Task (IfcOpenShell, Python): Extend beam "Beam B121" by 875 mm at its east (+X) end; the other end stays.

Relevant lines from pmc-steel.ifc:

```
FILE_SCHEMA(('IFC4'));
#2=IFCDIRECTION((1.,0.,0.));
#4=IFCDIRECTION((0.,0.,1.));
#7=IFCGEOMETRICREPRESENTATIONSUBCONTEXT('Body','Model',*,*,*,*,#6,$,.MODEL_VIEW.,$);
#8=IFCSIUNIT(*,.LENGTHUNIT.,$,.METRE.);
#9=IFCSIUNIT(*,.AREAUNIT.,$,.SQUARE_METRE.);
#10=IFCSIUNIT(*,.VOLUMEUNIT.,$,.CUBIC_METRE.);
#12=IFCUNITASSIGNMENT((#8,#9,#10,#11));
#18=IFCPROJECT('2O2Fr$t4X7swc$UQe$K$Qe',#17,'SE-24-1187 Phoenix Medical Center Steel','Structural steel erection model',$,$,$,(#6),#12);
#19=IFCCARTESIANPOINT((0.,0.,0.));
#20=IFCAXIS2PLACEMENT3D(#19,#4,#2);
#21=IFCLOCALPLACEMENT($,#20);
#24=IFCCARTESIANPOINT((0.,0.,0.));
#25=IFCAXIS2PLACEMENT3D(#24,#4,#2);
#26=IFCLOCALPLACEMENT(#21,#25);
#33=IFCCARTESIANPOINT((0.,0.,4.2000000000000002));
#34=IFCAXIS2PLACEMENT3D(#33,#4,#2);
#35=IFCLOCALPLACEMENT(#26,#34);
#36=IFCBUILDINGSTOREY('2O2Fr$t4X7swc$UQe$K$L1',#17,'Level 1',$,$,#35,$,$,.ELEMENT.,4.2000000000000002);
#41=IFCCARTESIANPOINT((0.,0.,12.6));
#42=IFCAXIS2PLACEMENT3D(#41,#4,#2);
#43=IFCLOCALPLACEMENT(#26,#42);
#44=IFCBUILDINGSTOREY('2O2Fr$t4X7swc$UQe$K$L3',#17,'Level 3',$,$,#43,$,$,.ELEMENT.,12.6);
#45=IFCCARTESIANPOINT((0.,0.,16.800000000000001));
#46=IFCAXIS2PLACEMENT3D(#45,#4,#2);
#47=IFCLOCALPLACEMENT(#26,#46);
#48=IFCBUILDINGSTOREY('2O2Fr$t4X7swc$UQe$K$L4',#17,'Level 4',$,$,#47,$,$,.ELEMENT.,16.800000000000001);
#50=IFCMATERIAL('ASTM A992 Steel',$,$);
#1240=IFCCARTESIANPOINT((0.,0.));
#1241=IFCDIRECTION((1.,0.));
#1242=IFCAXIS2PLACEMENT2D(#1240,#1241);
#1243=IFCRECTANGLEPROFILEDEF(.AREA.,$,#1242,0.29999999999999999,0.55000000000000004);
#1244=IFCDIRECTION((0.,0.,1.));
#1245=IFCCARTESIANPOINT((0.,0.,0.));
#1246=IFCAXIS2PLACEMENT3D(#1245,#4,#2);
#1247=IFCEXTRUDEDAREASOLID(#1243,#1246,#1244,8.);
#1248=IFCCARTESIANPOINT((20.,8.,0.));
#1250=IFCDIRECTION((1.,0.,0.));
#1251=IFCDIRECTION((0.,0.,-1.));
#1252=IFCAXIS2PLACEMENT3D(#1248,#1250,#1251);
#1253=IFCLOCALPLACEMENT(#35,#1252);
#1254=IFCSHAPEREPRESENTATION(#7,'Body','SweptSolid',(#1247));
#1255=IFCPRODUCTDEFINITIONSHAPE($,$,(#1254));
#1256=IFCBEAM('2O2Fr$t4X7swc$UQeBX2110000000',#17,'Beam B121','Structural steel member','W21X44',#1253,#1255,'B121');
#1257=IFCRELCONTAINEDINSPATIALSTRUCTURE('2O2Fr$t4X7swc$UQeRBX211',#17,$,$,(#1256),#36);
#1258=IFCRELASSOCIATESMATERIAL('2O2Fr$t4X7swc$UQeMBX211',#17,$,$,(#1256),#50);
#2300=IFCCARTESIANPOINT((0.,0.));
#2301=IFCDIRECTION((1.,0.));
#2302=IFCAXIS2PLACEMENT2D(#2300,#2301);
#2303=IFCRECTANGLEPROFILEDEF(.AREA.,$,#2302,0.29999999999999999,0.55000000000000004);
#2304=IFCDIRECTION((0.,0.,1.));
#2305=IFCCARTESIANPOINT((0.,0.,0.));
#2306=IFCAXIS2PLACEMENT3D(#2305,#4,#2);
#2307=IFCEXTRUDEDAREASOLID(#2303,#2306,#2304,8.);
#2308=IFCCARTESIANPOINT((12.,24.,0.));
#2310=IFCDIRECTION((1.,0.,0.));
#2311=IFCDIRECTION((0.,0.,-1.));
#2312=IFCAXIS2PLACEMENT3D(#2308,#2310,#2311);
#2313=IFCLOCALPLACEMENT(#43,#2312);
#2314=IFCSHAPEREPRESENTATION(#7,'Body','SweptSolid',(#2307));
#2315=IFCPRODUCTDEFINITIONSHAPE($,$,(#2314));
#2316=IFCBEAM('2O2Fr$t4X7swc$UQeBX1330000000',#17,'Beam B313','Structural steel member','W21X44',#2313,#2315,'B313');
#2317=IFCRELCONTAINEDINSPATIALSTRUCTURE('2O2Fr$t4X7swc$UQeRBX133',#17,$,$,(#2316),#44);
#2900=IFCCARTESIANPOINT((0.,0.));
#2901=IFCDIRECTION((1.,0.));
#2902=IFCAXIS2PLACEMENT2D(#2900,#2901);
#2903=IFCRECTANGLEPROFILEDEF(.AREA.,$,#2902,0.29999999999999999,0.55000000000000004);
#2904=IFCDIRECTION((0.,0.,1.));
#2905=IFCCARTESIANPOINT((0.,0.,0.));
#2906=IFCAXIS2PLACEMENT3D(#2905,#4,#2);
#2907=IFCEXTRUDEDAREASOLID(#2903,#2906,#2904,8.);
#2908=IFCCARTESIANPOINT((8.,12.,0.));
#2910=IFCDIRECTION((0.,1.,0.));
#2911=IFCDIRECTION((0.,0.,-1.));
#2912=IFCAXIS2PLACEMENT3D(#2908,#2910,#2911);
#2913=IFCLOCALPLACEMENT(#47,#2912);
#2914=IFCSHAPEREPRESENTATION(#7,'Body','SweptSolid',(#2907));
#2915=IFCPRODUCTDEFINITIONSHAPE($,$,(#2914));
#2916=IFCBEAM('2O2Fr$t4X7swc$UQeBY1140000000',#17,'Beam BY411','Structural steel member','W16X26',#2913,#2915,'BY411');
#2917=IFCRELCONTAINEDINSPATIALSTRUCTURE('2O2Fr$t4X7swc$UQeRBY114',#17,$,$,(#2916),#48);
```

```python
import ifcopenshell
import ifcopenshell.util.representation

model = ifcopenshell.open("pmc-steel.ifc")

member = model.by_guid("2O2Fr$t4X7swc$UQeBX2110000000")
change = 0.875

# The extrusion runs towards the end named, so only its depth changes.
body = ifcopenshell.util.representation.get_representation(member, "Model", "Body")
solid = body.Items[0]
old_length = solid.Depth
solid.Depth += change

print(f"length {old_length:g} -> {solid.Depth:g}")

model.write("pmc-steel_rev.ifc")
```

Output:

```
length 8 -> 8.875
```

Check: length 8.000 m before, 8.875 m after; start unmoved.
